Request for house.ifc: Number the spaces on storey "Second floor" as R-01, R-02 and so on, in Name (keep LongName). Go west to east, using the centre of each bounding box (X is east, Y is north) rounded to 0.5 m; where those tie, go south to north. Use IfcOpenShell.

First a look at what the model holds.

```python
import ifcopenshell
import ifcopenshell.util.element
import ifcopenshell.util.placement

model = ifcopenshell.open("house.ifc")
print(model.schema)
storey = next(s for s in model.by_type("IfcBuildingStorey") if s.Name == "Second floor")
spaces = [e for e in ifcopenshell.util.element.get_decomposition(storey) if e.is_a("IfcSpace")]
for e in sorted(spaces, key=lambda e: e.id()):
    origin = ifcopenshell.util.placement.get_local_placement(e.ObjectPlacement)[:3, 3]
    print(e.id(), e.Name, e.LongName, origin.round(2) + 0.0, sep=" | ")
```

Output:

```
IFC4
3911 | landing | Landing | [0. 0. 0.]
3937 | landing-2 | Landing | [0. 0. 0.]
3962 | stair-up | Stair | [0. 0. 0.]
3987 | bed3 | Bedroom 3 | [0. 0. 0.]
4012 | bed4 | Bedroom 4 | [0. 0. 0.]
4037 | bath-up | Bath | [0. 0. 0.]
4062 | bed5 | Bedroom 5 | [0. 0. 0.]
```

```python
import ifcopenshell
import ifcopenshell.geom
import ifcopenshell.util.element
import ifcopenshell.util.shape

model = ifcopenshell.open("house.ifc")
settings = ifcopenshell.geom.settings()
settings.set("use-world-coords", True)


def centre(element):
    shape = ifcopenshell.geom.create_shape(settings, element)
    return ifcopenshell.util.shape.get_bbox_centroid(shape.geometry)


storey = next(s for s in model.by_type("IfcBuildingStorey") if s.Name == "Second floor")
spaces = [e for e in ifcopenshell.util.element.get_decomposition(storey) if e.is_a("IfcSpace")]

# Insertion points can sit at a corner or the storey origin, so sort by the geometry (in metres).
centres = {e: centre(e) for e in spaces}
spaces.sort(key=lambda e: (round(centres[e][0] / 0.5), centres[e][1]))

for i, e in enumerate(spaces, start=1):
    number = f"R-{i:02d}"
    e.Name = number
    print(e.id(), number)

model.write("house_edited.ifc")
```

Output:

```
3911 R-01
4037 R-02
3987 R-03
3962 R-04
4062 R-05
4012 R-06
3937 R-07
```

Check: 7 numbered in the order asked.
